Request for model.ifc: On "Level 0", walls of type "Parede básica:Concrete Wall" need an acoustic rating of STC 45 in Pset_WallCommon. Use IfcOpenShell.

First a look at what the model holds.

```python
import ifcopenshell
import ifcopenshell.util.element

model = ifcopenshell.open("model.ifc")
print(model.schema)
storey = next(s for s in model.by_type("IfcBuildingStorey") if s.Name == "Level 0")
walls = [e for e in ifcopenshell.util.element.get_decomposition(storey) if e.is_a("IfcWall")]
seen = {}
for e in walls:
    element_type = ifcopenshell.util.element.get_type(e)
    key = (element_type.Name if element_type != e and element_type else None, ifcopenshell.util.element.get_pset(e, "Pset_WallCommon", "AcousticRating"))
    seen[key] = seen.get(key, 0) + 1
for (name, value), count in sorted(seen.items(), key=str):
    print(count, "x", name, "|", value)
```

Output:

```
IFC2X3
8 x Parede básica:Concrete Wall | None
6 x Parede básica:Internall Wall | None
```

```python
import ifcopenshell
import ifcopenshell.api.pset
import ifcopenshell.util.element

model = ifcopenshell.open("model.ifc")

storey = next(s for s in model.by_type("IfcBuildingStorey") if s.Name == "Level 0")
walls = [e for e in ifcopenshell.util.element.get_decomposition(storey) if e.is_a("IfcWall")]

count = 0
for e in walls:
    element_type = ifcopenshell.util.element.get_type(e)
    if element_type in (None, e) or element_type.Name != "Parede básica:Concrete Wall":
        continue
    # add_pset returns the element's existing set when there is one.
    pset = ifcopenshell.api.pset.add_pset(model, product=e, name="Pset_WallCommon")
    ifcopenshell.api.pset.edit_pset(model, pset=pset, properties={"AcousticRating": "STC 45"})
    count += 1

print(count, "walls updated")

model.write("model_rev.ifc")
```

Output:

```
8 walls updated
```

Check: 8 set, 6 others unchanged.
